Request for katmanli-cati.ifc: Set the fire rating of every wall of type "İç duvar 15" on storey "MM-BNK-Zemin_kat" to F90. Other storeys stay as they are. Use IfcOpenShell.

First a look at what the model holds.

```python
import ifcopenshell
import ifcopenshell.util.element

model = ifcopenshell.open("katmanli-cati.ifc")
print(model.schema)
storey = next(s for s in model.by_type("IfcBuildingStorey") if s.Name == "MM-BNK-Zemin_kat")
walls = [e for e in ifcopenshell.util.element.get_decomposition(storey) if e.is_a("IfcWall")]
seen = {}
for e in walls:
    element_type = ifcopenshell.util.element.get_type(e)
    key = (element_type.Name if element_type != e and element_type else None, ifcopenshell.util.element.get_pset(e, "Pset_WallCommon", "FireRating"))
    seen[key] = seen.get(key, 0) + 1
for (name, value), count in sorted(seen.items(), key=str):
    print(count, "x", name, "|", value)
```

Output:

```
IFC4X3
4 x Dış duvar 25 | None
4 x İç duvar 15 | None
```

```python
import ifcopenshell
import ifcopenshell.api.pset
import ifcopenshell.util.element

model = ifcopenshell.open("katmanli-cati.ifc")

storey = next(s for s in model.by_type("IfcBuildingStorey") if s.Name == "MM-BNK-Zemin_kat")
walls = [e for e in ifcopenshell.util.element.get_decomposition(storey) if e.is_a("IfcWall")]

count = 0
for e in walls:
    element_type = ifcopenshell.util.element.get_type(e)
    if element_type in (None, e) or element_type.Name != "İç duvar 15":
        continue
    # add_pset returns the element's existing set when there is one.
    pset = ifcopenshell.api.pset.add_pset(model, product=e, name="Pset_WallCommon")
    ifcopenshell.api.pset.edit_pset(model, pset=pset, properties={"FireRating": "F90"})
    count += 1

print(count, "walls updated")

model.write("katmanli-cati_updated.ifc")
```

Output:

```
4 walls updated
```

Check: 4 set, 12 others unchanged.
